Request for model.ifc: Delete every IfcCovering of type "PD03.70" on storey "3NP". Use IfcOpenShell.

First a look at what the model holds.

```python
import ifcopenshell
import ifcopenshell.util.element

model = ifcopenshell.open("model.ifc")
print(model.schema)
storey = next(s for s in model.by_type("IfcBuildingStorey") if s.Name == "3NP")
coverings = [e for e in ifcopenshell.util.element.get_decomposition(storey) if e.is_a("IfcCovering")]
seen = {}
for e in coverings:
    element_type = ifcopenshell.util.element.get_type(e)
    name = element_type.Name if element_type not in (None, e) else None
    seen[name] = seen.get(name, 0) + 1
for name, count in sorted(seen.items(), key=str):
    print(count, "x", name)
```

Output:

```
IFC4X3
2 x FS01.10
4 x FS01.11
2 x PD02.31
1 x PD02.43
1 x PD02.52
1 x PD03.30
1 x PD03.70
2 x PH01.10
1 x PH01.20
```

```python
import ifcopenshell
import ifcopenshell.api.root
import ifcopenshell.util.element

model = ifcopenshell.open("model.ifc")

storey = next(s for s in model.by_type("IfcBuildingStorey") if s.Name == "3NP")
coverings = [e for e in ifcopenshell.util.element.get_decomposition(storey) if e.is_a("IfcCovering")]
targets = [e for e in coverings if (t := ifcopenshell.util.element.get_type(e)) not in (None, e) and t.Name == "PD03.70"]

for e in targets:
    ifcopenshell.api.root.remove_product(model, product=e)
print(len(targets), "removed")

model.write("model_updated.ifc")
```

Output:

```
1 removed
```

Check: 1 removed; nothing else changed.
